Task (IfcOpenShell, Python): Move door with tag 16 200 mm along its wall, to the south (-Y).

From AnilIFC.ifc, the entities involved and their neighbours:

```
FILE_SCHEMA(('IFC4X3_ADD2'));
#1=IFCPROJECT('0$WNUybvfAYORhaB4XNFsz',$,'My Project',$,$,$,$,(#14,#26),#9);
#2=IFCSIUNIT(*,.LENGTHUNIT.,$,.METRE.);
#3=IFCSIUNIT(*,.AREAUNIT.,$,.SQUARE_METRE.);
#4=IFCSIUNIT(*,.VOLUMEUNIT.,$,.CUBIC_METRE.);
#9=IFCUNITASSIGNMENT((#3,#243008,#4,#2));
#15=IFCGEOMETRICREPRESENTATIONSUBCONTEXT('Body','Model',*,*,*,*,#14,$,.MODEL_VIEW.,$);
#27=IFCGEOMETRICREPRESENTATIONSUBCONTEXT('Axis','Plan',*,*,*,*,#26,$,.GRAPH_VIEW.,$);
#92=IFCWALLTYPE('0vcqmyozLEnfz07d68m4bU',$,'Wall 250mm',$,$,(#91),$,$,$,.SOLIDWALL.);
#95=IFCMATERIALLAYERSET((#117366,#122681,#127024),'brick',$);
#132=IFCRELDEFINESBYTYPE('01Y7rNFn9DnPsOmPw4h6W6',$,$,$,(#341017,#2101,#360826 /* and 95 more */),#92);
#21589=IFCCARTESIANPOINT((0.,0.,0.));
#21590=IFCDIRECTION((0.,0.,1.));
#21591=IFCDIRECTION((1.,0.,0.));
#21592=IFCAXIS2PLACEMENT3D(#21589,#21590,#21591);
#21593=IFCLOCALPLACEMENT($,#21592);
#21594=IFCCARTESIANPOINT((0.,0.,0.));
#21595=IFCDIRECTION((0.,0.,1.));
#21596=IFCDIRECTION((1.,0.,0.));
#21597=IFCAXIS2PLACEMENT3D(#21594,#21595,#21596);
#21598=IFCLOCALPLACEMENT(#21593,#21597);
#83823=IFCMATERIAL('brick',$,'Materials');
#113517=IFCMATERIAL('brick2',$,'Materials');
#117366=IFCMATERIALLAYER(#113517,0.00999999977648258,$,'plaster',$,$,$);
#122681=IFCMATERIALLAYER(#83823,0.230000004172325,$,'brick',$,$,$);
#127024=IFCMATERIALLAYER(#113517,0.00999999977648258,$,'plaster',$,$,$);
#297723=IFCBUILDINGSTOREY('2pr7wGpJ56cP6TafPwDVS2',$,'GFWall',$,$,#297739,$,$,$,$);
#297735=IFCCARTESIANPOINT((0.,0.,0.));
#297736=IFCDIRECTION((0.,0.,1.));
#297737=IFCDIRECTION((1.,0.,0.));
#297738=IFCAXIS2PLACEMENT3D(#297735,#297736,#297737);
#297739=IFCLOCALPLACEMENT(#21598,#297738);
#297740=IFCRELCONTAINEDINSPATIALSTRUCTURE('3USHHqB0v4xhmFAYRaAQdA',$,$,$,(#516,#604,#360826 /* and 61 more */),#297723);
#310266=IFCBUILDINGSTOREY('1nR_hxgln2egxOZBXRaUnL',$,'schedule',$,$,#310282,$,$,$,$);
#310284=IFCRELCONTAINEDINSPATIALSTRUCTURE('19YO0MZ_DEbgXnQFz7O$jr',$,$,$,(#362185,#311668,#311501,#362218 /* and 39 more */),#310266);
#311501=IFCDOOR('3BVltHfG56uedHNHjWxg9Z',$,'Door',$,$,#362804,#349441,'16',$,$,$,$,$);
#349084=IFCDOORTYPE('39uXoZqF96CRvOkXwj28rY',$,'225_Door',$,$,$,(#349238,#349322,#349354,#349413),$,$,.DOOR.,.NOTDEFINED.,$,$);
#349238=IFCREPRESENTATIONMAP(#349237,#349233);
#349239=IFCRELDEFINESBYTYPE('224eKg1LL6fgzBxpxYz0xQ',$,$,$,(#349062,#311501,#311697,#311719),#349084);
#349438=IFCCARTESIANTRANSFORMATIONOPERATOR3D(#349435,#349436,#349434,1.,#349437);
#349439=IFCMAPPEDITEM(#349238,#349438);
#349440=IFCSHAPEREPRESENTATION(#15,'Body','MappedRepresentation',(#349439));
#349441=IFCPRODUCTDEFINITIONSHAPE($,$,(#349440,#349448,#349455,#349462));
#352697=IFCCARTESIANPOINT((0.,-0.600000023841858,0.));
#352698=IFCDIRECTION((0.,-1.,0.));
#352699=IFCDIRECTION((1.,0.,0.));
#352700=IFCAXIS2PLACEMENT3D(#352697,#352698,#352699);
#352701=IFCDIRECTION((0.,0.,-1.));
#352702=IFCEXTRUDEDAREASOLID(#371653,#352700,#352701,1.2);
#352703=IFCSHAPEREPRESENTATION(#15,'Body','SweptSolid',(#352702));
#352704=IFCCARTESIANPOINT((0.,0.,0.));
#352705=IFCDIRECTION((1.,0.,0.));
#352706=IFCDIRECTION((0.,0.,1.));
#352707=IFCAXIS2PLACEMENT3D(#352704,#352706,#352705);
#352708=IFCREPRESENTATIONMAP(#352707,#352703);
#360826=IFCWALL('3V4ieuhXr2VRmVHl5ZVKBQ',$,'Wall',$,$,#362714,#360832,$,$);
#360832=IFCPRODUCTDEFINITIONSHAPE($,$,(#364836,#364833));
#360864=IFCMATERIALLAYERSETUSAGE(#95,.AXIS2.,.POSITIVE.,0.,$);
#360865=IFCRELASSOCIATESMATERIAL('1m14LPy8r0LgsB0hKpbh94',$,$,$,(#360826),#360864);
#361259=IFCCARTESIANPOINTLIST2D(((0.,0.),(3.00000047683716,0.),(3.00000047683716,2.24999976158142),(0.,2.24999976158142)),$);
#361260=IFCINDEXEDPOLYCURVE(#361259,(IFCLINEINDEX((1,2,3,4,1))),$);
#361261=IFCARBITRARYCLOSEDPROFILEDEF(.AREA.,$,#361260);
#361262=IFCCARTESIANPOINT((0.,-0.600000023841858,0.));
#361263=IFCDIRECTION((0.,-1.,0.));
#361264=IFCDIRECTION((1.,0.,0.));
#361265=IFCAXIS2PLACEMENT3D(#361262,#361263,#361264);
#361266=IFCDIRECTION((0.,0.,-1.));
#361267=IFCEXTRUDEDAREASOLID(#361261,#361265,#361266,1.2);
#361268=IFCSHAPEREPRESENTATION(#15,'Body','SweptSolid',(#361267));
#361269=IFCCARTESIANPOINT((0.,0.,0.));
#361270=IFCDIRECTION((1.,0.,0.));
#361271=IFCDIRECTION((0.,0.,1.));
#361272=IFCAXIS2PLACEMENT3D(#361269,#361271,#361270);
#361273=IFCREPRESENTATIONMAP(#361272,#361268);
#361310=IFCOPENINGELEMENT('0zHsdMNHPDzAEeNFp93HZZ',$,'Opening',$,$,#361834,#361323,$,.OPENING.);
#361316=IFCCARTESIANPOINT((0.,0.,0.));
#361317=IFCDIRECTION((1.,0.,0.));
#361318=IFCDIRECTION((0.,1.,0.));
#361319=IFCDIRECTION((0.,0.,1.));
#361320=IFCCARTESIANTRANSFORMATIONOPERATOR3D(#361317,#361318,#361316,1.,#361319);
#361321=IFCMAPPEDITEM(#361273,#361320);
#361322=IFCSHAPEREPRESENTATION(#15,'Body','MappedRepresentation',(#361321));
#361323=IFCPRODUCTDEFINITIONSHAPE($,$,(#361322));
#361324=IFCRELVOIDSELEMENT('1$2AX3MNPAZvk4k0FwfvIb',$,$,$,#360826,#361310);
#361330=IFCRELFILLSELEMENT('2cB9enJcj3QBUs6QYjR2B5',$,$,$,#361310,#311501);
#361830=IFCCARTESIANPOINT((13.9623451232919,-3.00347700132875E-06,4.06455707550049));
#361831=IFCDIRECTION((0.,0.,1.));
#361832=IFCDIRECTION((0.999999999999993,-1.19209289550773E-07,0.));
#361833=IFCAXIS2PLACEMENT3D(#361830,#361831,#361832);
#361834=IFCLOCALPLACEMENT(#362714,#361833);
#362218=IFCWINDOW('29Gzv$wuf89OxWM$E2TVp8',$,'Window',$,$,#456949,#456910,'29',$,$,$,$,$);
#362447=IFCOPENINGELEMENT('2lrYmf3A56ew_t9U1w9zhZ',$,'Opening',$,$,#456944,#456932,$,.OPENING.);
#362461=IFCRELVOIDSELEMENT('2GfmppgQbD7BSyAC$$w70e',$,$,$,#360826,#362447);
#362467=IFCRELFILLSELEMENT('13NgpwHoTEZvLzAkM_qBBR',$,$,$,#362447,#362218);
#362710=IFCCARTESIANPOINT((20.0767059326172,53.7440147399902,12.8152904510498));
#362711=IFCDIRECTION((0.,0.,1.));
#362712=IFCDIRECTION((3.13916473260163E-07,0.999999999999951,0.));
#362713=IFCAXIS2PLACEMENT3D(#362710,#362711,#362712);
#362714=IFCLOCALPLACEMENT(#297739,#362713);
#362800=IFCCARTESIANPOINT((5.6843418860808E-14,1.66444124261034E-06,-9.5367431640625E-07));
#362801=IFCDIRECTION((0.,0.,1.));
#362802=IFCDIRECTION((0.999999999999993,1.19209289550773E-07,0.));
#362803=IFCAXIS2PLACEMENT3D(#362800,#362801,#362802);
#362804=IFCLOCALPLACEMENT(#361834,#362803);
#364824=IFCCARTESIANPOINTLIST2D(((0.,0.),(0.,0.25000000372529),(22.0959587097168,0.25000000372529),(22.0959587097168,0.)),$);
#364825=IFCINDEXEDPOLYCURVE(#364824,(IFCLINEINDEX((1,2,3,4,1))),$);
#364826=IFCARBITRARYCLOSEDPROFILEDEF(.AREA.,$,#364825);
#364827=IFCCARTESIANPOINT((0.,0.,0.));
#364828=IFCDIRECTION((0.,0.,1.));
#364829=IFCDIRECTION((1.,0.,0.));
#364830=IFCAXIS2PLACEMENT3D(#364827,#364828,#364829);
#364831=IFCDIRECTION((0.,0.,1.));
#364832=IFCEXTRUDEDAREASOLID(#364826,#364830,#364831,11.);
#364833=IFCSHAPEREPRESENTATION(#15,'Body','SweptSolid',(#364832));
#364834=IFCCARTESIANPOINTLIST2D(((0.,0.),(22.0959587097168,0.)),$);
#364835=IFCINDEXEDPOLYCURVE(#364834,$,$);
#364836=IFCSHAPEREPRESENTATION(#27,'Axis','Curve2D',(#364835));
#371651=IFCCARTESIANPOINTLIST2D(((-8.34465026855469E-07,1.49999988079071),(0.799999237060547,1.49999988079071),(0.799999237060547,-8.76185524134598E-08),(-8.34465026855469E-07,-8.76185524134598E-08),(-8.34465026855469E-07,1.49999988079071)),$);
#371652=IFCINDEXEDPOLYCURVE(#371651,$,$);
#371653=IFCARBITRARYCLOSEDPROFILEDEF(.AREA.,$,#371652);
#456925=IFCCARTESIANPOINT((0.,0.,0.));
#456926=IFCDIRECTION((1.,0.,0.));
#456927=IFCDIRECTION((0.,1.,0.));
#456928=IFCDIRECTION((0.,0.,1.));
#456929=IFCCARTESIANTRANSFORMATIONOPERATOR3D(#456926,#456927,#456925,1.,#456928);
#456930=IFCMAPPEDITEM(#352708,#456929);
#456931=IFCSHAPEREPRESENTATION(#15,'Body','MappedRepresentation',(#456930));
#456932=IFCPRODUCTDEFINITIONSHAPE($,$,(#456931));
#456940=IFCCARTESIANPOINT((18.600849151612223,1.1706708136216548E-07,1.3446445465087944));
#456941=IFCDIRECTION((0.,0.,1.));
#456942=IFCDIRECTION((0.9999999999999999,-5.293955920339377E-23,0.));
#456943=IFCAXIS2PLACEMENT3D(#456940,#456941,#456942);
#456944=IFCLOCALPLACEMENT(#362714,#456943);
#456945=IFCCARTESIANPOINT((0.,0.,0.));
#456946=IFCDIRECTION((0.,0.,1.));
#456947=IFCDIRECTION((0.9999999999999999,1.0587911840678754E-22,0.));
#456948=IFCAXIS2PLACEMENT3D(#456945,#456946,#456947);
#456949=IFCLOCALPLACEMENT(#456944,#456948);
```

```python
import ifcopenshell
import ifcopenshell.api.geometry
import ifcopenshell.util.placement

model = ifcopenshell.open("AnilIFC.ifc")

door = model.by_guid("3BVltHfG56uedHNHjWxg9Z")
opening = door.FillsVoids[0].RelatingOpeningElement
wall = opening.VoidsElements[0].RelatingBuildingElement

wall_matrix = ifcopenshell.util.placement.get_local_placement(wall.ObjectPlacement)
shift = wall_matrix[:3, 0] * -0.2
before = ifcopenshell.util.placement.get_local_placement(door.ObjectPlacement)[:3, 3].copy()

# The door is placed relative to its opening, so it follows when the opening moves.
matrix = ifcopenshell.util.placement.get_local_placement(opening.ObjectPlacement)
matrix[:3, 3] += shift
ifcopenshell.api.geometry.edit_object_placement(
    model, product=opening, matrix=matrix, is_si=False, should_transform_children=True
)

after = ifcopenshell.util.placement.get_local_placement(door.ObjectPlacement)[:3, 3]
print("door moved by", (after - before).round(3) + 0.0)

model.write("AnilIFC_v2.ifc")
```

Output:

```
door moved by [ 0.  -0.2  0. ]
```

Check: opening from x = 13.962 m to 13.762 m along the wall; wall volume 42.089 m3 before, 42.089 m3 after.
